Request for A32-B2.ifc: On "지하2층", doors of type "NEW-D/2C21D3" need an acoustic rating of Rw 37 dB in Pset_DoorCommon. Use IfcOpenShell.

First a look at what the model holds.

```python
import ifcopenshell
import ifcopenshell.util.element

model = ifcopenshell.open("A32-B2.ifc")
print(model.schema)
storey = next(s for s in model.by_type("IfcBuildingStorey") if s.Name == "지하2층")
doors = [e for e in ifcopenshell.util.element.get_decomposition(storey) if e.is_a("IfcDoor")]
seen = {}
for e in doors:
    element_type = ifcopenshell.util.element.get_type(e)
    key = (element_type.Name if element_type != e and element_type else None, ifcopenshell.util.element.get_pset(e, "Pset_DoorCommon", "AcousticRating"))
    seen[key] = seen.get(key, 0) + 1
for (name, value), count in sorted(seen.items(), key=str):
    print(count, "x", name, "|", value)
```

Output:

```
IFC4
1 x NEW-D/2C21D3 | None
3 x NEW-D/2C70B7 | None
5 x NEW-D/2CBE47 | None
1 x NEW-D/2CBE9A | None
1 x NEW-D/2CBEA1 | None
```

```python
import ifcopenshell
import ifcopenshell.api.pset
import ifcopenshell.util.element

model = ifcopenshell.open("A32-B2.ifc")

storey = next(s for s in model.by_type("IfcBuildingStorey") if s.Name == "지하2층")
doors = [e for e in ifcopenshell.util.element.get_decomposition(storey) if e.is_a("IfcDoor")]

count = 0
for e in doors:
    element_type = ifcopenshell.util.element.get_type(e)
    if element_type in (None, e) or element_type.Name != "NEW-D/2C21D3":
        continue
    # add_pset returns the element's existing set when there is one.
    pset = ifcopenshell.api.pset.add_pset(model, product=e, name="Pset_DoorCommon")
    ifcopenshell.api.pset.edit_pset(model, pset=pset, properties={"AcousticRating": "Rw 37 dB"})
    count += 1

print(count, "doors updated")

model.write("A32-B2_updated.ifc")
```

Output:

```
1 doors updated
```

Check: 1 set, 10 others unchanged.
